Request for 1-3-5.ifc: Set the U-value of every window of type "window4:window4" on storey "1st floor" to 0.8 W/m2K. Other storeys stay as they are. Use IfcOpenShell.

First a look at what the model holds.

```python
import ifcopenshell
import ifcopenshell.util.element

model = ifcopenshell.open("1-3-5.ifc")
print(model.schema)
storey = next(s for s in model.by_type("IfcBuildingStorey") if s.Name == "1st floor")
windows = [e for e in ifcopenshell.util.element.get_decomposition(storey) if e.is_a("IfcWindow")]
seen = {}
for e in windows:
    element_type = ifcopenshell.util.element.get_type(e)
    key = (element_type.Name if element_type != e and element_type else None, ifcopenshell.util.element.get_pset(e, "Pset_WindowCommon", "ThermalTransmittance"))
    seen[key] = seen.get(key, 0) + 1
for (name, value), count in sorted(seen.items(), key=str):
    print(count, "x", name, "|", value)
```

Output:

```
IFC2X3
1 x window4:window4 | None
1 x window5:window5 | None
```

```python
import ifcopenshell
import ifcopenshell.api.pset
import ifcopenshell.util.element

model = ifcopenshell.open("1-3-5.ifc")

storey = next(s for s in model.by_type("IfcBuildingStorey") if s.Name == "1st floor")
windows = [e for e in ifcopenshell.util.element.get_decomposition(storey) if e.is_a("IfcWindow")]

count = 0
for e in windows:
    element_type = ifcopenshell.util.element.get_type(e)
    if element_type in (None, e) or element_type.Name != "window4:window4":
        continue
    # add_pset returns the element's existing set when there is one.
    pset = ifcopenshell.api.pset.add_pset(model, product=e, name="Pset_WindowCommon")
    ifcopenshell.api.pset.edit_pset(model, pset=pset, properties={"ThermalTransmittance": 0.8})
    count += 1

print(count, "windows updated")

model.write("1-3-5_v2.ifc")
```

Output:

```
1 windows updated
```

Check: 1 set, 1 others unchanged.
